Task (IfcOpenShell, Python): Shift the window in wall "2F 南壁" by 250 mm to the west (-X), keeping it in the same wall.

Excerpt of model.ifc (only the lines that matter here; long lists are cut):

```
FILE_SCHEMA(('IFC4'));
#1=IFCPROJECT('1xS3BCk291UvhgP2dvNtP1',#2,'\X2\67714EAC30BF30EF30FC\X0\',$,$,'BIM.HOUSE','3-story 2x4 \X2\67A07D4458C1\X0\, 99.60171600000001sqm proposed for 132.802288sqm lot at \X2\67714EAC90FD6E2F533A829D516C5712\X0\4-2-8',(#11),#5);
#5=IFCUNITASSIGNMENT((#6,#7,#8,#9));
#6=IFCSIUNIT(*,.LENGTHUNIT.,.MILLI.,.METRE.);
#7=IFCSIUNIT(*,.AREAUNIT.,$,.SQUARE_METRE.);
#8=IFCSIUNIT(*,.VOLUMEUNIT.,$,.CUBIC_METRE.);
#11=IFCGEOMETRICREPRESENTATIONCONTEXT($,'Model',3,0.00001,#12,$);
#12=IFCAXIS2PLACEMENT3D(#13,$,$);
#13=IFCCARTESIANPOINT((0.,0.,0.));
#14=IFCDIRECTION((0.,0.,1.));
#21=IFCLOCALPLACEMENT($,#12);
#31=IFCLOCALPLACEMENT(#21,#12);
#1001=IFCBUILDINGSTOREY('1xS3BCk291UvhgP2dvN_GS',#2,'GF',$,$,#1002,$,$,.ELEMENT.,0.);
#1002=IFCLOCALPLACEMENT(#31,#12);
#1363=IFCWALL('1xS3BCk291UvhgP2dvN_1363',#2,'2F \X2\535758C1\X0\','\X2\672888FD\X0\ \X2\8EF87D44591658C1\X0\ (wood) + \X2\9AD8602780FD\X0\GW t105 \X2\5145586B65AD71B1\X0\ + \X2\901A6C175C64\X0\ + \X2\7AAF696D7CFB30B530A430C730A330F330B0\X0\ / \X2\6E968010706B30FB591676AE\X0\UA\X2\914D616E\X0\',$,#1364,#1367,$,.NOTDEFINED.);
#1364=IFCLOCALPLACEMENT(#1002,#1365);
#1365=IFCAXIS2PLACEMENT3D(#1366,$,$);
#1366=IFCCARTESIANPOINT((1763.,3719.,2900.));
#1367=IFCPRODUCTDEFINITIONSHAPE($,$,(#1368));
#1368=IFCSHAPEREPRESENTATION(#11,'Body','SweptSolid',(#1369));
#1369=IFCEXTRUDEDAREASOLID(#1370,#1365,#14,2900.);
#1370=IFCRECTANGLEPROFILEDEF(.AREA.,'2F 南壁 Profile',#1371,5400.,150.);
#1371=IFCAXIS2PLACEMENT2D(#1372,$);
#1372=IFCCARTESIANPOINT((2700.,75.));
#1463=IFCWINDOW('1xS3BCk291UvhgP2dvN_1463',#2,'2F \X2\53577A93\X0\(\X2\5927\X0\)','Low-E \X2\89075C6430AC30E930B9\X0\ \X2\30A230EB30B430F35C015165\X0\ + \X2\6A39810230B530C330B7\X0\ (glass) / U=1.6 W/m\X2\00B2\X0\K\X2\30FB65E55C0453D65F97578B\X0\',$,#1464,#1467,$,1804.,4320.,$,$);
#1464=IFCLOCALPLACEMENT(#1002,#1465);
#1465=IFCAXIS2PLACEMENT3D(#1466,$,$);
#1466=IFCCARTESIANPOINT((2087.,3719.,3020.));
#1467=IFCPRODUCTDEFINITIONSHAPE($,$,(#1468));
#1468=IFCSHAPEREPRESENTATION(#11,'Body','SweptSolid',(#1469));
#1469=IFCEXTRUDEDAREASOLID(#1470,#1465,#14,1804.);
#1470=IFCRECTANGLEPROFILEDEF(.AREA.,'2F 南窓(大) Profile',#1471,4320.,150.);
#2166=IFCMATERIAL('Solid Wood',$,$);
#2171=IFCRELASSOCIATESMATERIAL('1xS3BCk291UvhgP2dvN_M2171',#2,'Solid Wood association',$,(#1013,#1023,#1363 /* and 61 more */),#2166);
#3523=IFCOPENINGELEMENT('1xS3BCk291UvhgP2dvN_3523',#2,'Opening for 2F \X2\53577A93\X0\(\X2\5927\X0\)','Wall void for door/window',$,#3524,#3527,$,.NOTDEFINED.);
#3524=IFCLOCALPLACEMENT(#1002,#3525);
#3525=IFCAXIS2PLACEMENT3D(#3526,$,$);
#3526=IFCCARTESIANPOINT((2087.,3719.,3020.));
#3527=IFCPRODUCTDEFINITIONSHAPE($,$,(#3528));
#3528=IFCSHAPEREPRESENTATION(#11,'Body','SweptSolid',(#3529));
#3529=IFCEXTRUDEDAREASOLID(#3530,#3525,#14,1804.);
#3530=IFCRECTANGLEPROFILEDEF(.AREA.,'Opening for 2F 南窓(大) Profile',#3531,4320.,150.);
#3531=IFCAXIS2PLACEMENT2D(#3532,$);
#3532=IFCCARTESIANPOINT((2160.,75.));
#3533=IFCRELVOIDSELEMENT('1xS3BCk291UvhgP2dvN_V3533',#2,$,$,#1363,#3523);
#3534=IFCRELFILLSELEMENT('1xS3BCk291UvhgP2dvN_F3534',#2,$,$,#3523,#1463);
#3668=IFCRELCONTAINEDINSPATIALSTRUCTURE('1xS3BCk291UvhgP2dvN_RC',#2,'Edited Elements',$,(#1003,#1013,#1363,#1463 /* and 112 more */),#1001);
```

```python
import ifcopenshell
import ifcopenshell.api.geometry
import ifcopenshell.util.placement

model = ifcopenshell.open("model.ifc")

window = model.by_guid("1xS3BCk291UvhgP2dvN_1463")
opening = window.FillsVoids[0].RelatingOpeningElement
wall = opening.VoidsElements[0].RelatingBuildingElement

wall_matrix = ifcopenshell.util.placement.get_local_placement(wall.ObjectPlacement)
shift = wall_matrix[:3, 0] * -250.0
before = ifcopenshell.util.placement.get_local_placement(window.ObjectPlacement)[:3, 3].copy()

# The window is not placed relative to its opening, so move both.
for product in (opening, window):
    matrix = ifcopenshell.util.placement.get_local_placement(product.ObjectPlacement)
    matrix[:3, 3] += shift
    ifcopenshell.api.geometry.edit_object_placement(model, product=product, matrix=matrix, is_si=False)

after = ifcopenshell.util.placement.get_local_placement(window.ObjectPlacement)[:3, 3]
print("window moved by", (after - before).round(3) + 0.0)

model.write("model-out.ifc")
```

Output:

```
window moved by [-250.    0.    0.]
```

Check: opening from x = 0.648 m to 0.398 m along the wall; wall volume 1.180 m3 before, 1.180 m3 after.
